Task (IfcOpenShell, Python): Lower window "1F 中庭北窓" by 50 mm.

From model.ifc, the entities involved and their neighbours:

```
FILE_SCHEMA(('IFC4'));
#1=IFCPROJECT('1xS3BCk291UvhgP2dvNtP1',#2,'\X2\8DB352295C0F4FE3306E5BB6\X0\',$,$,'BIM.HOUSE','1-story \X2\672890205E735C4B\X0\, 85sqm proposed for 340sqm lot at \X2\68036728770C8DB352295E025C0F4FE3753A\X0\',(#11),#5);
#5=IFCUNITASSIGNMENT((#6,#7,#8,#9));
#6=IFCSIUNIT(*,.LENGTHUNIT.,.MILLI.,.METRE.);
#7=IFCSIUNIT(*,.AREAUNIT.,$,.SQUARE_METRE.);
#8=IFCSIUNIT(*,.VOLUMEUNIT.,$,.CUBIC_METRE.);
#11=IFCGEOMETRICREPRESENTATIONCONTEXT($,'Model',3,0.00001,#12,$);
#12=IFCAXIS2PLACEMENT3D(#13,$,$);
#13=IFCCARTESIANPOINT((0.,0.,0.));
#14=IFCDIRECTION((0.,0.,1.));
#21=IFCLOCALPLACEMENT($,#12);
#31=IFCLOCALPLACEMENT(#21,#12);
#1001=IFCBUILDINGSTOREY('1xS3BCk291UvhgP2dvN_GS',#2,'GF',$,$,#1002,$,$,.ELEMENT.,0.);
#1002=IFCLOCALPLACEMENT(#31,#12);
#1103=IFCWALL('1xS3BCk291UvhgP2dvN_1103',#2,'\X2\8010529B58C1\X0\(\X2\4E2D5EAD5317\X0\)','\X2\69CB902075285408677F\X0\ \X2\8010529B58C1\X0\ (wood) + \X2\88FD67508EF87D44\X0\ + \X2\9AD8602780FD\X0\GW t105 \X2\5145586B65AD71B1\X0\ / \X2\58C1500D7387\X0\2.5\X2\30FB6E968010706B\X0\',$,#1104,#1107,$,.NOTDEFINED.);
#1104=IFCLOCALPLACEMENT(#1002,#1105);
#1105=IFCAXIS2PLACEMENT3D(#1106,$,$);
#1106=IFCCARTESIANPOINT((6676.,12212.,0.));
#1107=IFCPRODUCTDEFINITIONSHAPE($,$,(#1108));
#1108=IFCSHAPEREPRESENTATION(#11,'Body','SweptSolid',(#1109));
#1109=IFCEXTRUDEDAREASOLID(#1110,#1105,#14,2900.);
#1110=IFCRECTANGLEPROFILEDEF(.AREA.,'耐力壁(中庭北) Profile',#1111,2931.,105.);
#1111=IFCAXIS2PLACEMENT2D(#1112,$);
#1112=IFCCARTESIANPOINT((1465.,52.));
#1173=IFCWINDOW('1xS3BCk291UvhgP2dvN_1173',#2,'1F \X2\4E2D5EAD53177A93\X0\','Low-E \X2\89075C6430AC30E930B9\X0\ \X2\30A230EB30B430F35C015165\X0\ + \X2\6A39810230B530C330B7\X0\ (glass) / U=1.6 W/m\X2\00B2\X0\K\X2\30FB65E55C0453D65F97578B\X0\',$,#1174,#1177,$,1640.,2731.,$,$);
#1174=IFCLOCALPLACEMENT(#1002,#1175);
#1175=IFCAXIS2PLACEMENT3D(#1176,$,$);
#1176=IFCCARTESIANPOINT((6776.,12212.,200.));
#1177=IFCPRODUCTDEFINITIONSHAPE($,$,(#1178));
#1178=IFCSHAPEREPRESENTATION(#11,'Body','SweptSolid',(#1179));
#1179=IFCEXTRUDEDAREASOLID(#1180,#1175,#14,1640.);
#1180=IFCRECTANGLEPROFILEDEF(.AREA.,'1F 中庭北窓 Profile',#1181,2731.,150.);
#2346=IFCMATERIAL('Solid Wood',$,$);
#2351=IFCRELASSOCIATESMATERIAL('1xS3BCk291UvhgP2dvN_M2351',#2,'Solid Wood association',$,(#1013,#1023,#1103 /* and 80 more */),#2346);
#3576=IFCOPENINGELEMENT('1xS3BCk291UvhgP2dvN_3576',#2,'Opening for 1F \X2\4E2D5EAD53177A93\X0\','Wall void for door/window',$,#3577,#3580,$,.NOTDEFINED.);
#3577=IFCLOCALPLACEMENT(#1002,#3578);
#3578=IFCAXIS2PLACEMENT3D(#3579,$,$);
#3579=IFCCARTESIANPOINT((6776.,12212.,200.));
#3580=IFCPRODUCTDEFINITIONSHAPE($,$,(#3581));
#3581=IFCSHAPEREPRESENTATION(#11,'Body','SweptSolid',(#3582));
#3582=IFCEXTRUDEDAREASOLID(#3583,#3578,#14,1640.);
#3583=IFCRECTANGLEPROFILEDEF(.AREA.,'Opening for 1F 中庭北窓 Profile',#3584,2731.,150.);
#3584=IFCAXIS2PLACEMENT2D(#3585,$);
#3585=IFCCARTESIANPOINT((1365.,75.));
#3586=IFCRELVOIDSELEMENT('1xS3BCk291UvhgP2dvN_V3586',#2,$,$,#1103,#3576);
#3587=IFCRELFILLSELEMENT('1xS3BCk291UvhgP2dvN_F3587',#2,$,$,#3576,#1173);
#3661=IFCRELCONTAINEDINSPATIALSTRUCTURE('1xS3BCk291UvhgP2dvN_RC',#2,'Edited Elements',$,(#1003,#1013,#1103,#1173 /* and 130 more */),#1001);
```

```python
import numpy as np
import ifcopenshell
import ifcopenshell.api.geometry
import ifcopenshell.util.placement
import ifcopenshell.util.unit

model = ifcopenshell.open("model.ifc")
unit_scale = ifcopenshell.util.unit.calculate_unit_scale(model)

window = model.by_guid("1xS3BCk291UvhgP2dvN_1173")
opening = window.FillsVoids[0].RelatingOpeningElement
dz = -0.05 / unit_scale

shift = np.array([0.0, 0.0, dz])
# The window is not placed relative to its opening, so move both.
for product in (opening, window):
    matrix = ifcopenshell.util.placement.get_local_placement(product.ObjectPlacement)
    matrix[:3, 3] += shift
    ifcopenshell.api.geometry.edit_object_placement(model, product=product, matrix=matrix, is_si=False)

print(f"moved by {dz * unit_scale:+.3f} m")

model.write("model-out.ifc")
```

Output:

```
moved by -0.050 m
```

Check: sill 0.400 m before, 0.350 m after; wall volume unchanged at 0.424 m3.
